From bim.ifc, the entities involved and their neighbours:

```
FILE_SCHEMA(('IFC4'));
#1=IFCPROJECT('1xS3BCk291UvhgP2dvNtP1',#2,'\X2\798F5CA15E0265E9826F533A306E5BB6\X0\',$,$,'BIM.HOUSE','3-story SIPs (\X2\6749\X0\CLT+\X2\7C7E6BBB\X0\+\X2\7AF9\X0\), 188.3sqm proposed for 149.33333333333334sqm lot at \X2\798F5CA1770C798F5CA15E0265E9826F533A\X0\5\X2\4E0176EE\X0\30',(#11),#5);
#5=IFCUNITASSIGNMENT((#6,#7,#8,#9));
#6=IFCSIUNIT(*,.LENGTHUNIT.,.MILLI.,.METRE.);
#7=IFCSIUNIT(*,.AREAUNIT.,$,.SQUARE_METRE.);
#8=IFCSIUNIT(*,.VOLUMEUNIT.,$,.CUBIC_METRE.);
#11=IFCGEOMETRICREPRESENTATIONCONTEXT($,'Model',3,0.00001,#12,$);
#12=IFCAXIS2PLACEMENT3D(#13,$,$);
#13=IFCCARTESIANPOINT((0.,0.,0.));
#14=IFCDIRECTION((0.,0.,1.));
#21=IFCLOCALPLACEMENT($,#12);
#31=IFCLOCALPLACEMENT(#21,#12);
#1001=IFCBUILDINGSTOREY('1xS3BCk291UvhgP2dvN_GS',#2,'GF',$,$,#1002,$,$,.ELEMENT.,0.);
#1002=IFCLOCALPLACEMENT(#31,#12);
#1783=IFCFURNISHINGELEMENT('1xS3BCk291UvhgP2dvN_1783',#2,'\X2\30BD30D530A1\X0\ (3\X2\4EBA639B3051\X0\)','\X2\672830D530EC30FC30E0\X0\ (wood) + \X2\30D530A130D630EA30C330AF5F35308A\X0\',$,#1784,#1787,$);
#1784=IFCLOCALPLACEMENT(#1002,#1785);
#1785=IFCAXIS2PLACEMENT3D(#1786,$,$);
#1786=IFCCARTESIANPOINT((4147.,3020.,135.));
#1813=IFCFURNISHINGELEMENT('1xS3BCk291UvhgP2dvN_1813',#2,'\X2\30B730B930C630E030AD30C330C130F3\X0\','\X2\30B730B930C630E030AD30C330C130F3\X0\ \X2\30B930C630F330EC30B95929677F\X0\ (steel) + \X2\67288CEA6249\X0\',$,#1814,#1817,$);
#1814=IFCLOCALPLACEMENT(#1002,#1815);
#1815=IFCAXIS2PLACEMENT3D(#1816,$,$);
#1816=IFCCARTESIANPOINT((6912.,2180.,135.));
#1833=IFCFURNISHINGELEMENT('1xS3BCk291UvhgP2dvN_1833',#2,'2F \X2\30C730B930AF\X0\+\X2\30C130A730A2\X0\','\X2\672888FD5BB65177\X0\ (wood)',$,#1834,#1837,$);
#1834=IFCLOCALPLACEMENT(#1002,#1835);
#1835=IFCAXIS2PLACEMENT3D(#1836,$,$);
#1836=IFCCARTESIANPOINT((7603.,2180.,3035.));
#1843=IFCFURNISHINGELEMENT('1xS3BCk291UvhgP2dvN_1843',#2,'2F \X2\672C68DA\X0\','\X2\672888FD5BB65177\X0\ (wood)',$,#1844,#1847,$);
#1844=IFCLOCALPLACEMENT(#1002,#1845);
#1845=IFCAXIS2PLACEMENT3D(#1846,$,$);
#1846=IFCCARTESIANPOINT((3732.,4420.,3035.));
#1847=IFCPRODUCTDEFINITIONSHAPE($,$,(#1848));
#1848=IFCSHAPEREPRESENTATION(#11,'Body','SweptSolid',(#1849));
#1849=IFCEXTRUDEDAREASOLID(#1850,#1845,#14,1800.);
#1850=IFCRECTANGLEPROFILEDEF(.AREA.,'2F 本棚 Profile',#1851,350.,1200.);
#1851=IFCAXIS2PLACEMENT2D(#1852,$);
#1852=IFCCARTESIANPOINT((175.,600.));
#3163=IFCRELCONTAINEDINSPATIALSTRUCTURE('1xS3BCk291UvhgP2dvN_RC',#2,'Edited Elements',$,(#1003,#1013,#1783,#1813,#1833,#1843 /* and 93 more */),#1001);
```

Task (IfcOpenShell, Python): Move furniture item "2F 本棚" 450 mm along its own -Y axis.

```python
import ifcopenshell
import ifcopenshell.api.geometry
import ifcopenshell.util.placement
import ifcopenshell.util.unit

model = ifcopenshell.open("bim.ifc")
unit_scale = ifcopenshell.util.unit.calculate_unit_scale(model)

item = model.by_guid("1xS3BCk291UvhgP2dvN_1843")
matrix = ifcopenshell.util.placement.get_local_placement(item.ObjectPlacement)
matrix[:3, 3] -= matrix[:3, 1] * 0.45 / unit_scale
ifcopenshell.api.geometry.edit_object_placement(model, product=item, matrix=matrix, is_si=False)

print(ifcopenshell.util.placement.get_local_placement(item.ObjectPlacement).round(3) + 0.0)

model.write("bim-out.ifc")
```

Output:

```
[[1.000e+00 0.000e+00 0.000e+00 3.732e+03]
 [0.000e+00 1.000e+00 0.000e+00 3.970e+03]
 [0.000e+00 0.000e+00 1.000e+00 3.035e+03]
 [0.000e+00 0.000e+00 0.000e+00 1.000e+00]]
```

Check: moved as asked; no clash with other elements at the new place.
